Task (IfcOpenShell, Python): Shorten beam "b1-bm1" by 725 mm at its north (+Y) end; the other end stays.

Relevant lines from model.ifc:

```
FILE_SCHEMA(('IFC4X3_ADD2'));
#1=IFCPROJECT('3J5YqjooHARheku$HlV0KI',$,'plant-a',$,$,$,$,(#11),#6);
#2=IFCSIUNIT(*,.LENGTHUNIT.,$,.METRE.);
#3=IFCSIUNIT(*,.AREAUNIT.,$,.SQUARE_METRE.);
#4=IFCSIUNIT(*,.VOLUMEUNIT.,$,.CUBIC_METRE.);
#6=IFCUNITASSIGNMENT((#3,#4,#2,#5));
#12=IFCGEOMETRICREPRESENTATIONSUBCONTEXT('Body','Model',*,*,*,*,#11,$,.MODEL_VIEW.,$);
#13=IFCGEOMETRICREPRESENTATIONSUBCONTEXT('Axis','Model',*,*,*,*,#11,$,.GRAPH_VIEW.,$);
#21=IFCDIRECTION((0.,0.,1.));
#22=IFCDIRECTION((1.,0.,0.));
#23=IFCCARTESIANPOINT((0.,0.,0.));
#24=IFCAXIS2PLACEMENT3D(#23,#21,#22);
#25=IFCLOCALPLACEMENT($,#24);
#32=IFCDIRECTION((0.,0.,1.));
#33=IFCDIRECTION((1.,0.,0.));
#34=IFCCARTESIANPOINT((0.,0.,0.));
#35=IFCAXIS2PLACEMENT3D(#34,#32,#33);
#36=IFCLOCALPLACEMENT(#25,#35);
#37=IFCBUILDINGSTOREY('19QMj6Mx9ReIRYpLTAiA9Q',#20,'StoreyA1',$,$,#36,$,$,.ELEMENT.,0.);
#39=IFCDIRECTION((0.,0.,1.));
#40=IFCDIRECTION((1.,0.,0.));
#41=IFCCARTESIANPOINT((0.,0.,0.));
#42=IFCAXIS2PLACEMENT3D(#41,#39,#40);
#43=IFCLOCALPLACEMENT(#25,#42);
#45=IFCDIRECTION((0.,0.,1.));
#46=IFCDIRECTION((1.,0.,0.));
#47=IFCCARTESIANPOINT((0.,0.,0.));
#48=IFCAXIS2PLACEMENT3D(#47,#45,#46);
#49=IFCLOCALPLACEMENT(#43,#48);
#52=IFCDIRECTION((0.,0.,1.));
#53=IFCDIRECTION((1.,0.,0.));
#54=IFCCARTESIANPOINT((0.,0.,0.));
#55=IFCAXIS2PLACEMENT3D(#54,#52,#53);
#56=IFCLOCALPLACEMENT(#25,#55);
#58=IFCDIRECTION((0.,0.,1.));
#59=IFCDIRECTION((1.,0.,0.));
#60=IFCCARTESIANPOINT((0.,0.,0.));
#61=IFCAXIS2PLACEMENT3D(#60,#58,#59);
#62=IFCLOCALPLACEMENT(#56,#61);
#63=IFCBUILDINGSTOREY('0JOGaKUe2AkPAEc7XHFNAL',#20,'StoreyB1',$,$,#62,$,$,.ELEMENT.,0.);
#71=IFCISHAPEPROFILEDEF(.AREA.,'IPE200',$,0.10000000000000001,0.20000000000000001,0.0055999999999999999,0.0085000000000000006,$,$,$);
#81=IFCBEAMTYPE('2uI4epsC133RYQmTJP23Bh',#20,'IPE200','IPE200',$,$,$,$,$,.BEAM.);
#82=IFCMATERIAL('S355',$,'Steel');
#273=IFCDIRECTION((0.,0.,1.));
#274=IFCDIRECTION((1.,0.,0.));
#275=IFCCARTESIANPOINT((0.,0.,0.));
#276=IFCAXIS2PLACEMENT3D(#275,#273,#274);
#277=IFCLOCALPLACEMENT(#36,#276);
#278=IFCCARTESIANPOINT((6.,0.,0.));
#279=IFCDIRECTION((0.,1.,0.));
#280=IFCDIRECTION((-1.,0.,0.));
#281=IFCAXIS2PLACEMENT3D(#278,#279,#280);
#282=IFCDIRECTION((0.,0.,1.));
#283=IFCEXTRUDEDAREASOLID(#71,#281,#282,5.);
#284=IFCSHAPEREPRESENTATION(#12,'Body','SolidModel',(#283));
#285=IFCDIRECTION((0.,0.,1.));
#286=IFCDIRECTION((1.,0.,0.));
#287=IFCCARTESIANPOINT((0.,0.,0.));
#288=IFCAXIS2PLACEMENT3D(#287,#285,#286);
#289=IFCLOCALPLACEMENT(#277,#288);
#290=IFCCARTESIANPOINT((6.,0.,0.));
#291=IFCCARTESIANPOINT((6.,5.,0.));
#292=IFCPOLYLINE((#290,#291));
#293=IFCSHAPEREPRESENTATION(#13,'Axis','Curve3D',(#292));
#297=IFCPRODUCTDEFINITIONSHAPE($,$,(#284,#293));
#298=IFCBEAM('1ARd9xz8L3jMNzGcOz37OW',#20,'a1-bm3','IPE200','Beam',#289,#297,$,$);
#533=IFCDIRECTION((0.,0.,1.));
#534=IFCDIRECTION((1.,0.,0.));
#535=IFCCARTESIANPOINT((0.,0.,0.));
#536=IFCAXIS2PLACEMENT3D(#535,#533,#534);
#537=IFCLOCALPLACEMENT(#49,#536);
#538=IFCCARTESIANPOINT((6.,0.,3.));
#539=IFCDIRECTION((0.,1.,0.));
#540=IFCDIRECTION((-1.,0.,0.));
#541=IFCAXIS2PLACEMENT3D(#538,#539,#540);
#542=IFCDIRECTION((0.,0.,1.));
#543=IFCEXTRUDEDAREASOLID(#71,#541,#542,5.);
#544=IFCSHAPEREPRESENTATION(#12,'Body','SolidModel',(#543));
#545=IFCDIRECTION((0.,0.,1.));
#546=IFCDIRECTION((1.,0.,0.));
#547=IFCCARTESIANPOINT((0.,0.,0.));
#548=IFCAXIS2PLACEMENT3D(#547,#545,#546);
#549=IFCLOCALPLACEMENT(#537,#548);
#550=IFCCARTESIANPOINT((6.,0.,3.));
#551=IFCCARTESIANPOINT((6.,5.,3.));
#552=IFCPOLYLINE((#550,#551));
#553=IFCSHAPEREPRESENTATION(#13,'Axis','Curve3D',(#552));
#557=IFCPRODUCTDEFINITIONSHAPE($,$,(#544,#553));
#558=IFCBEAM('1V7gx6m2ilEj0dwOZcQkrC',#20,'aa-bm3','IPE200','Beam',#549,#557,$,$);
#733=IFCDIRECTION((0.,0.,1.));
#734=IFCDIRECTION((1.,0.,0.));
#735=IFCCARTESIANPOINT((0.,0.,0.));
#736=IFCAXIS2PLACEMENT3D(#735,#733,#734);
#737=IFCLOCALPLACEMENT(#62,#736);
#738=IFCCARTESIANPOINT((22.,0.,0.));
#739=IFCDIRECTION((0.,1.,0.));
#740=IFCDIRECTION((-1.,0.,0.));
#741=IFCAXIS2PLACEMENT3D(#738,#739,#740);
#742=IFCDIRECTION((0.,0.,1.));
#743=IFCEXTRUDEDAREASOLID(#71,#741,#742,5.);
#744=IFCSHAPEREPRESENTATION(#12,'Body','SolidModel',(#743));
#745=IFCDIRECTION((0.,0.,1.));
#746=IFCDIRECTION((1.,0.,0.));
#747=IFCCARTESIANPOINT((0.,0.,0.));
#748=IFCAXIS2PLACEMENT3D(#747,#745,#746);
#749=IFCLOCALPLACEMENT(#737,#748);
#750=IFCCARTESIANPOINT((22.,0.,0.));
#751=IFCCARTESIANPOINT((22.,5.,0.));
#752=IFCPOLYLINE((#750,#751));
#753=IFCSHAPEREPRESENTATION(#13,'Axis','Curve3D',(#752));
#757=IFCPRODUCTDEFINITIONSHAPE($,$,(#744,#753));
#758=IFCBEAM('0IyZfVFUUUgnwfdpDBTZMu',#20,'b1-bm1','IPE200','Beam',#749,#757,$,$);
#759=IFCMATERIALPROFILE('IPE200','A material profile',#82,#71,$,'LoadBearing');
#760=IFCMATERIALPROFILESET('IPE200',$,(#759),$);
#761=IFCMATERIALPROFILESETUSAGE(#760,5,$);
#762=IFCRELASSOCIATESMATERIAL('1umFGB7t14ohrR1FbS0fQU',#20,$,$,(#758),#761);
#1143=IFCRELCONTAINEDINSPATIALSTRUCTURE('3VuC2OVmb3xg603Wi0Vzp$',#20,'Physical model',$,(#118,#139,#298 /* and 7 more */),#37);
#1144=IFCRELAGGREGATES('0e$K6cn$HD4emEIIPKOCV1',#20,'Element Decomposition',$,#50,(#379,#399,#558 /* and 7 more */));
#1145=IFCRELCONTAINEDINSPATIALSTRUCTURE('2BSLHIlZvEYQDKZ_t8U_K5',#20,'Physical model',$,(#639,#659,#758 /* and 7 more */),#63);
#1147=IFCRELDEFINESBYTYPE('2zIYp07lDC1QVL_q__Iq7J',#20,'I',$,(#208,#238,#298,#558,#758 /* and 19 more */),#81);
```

```python
import numpy as np
import ifcopenshell
import ifcopenshell.util.representation
import ifcopenshell.util.unit

model = ifcopenshell.open("model.ifc")
unit_scale = ifcopenshell.util.unit.calculate_unit_scale(model)

member = model.by_guid("0IyZfVFUUUgnwfdpDBTZMu")
change = -0.725 / unit_scale

# The extrusion runs towards the end named, so only its depth changes.
body = ifcopenshell.util.representation.get_representation(member, "Model", "Body")
solid = body.Items[0]
old_length = solid.Depth
solid.Depth += change

# Move the axis end point with it.
axis = next(r for r in member.Representation.Representations if r.RepresentationIdentifier == "Axis").Items[0]
start, end = (np.array(p.Coordinates) for p in axis.Points)
end = end + (end - start) / np.linalg.norm(end - start) * change
point = model.createIfcCartesianPoint(end.tolist())
axis.Points = [axis.Points[0], point]

print(f"length {old_length:g} -> {solid.Depth:g}")

model.write("model_updated.ifc")
```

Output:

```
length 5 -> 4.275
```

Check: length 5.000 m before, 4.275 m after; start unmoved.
